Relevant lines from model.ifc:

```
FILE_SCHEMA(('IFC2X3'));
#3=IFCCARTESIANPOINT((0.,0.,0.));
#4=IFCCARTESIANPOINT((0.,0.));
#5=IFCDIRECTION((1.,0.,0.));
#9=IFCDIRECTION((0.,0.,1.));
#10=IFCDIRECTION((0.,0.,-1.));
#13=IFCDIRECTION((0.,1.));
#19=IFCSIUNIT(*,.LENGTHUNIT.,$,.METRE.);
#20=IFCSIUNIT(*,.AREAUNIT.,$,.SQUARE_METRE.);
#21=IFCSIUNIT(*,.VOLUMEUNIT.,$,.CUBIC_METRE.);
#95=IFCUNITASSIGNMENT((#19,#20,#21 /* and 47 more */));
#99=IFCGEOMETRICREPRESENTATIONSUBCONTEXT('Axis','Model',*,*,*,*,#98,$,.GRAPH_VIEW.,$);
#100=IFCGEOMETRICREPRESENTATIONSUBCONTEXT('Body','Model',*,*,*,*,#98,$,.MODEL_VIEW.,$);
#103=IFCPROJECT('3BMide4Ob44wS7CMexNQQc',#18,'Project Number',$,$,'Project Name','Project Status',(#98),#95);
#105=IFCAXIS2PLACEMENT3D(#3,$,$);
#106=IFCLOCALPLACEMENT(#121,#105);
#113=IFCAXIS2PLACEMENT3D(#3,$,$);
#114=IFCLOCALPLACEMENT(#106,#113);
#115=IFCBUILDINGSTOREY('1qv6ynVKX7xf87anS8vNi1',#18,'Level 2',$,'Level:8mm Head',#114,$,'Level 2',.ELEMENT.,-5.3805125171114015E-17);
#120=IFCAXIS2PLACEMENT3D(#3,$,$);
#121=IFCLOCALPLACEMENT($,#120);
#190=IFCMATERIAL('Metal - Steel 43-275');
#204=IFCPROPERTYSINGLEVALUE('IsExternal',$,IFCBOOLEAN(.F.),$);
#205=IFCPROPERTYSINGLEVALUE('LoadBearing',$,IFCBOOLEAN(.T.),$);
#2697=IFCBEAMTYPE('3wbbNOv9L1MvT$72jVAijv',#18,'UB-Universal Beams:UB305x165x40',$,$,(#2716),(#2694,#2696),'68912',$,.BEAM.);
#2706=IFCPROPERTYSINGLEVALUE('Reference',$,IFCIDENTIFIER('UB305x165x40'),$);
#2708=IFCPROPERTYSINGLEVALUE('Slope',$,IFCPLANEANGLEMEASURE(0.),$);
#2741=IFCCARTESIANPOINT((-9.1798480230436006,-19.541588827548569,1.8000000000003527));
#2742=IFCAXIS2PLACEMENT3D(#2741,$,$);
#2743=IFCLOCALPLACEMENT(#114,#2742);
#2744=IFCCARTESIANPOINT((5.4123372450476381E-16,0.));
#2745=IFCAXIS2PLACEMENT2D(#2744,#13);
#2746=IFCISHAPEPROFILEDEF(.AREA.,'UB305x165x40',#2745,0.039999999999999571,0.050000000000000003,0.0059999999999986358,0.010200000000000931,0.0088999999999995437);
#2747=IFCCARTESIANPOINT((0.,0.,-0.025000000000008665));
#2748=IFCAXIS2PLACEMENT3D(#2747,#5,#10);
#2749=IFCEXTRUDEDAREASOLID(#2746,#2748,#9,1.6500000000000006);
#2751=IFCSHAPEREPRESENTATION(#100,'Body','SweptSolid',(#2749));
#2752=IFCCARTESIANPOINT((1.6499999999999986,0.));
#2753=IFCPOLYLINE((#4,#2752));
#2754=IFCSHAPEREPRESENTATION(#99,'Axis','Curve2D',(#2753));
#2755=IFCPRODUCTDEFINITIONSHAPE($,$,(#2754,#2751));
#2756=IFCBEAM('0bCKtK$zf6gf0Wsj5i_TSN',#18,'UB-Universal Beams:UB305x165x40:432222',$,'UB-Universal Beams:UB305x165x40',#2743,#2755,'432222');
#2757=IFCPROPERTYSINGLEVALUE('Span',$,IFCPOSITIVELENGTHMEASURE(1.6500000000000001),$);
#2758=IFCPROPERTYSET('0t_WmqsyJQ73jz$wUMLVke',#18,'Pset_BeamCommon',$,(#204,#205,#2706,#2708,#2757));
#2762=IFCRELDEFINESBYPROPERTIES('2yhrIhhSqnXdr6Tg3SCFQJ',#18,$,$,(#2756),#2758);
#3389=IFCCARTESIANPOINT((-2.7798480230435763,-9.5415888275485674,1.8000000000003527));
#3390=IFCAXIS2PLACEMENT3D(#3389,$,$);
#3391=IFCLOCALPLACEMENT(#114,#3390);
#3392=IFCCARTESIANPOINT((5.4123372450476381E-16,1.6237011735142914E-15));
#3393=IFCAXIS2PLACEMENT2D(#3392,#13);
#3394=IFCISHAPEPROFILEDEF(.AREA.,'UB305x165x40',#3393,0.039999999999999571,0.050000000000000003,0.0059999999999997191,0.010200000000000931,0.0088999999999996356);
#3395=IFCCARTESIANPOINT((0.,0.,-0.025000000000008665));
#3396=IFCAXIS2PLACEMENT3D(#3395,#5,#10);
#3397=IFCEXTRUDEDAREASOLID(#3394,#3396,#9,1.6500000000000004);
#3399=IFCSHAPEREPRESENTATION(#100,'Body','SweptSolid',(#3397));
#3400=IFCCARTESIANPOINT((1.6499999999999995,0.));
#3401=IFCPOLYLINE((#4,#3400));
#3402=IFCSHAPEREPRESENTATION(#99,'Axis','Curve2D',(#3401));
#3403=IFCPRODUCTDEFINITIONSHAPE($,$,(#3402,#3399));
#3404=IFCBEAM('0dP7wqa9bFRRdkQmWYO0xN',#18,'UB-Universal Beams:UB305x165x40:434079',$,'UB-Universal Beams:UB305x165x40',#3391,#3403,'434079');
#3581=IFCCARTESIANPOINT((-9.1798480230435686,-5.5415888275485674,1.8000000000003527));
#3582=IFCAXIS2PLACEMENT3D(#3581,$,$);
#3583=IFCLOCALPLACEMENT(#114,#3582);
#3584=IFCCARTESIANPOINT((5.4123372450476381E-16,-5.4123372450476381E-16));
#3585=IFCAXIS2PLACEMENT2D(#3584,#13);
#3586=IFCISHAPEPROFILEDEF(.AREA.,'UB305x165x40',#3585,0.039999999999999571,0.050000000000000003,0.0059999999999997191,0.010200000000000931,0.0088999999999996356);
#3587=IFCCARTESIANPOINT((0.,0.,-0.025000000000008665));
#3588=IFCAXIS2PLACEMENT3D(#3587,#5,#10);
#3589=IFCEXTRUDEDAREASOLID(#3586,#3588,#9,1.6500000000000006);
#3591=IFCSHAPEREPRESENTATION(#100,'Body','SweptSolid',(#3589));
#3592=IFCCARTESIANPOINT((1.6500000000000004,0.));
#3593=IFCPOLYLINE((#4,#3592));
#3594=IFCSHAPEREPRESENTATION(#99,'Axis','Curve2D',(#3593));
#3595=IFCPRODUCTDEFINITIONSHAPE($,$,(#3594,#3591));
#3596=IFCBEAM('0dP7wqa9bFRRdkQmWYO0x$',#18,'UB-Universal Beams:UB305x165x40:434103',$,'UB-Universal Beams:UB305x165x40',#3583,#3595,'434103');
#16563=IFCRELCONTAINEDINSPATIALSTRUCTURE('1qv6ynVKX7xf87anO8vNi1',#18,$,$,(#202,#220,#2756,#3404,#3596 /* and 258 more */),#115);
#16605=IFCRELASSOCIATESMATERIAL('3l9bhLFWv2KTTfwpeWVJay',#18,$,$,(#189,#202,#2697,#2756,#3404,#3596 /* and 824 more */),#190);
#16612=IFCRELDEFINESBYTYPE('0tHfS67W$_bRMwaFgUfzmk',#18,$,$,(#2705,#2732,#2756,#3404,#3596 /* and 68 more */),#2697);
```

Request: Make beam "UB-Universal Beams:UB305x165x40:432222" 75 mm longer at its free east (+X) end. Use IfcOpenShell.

```python
import numpy as np
import ifcopenshell
import ifcopenshell.api.pset
import ifcopenshell.util.element
import ifcopenshell.util.representation
import ifcopenshell.util.unit

model = ifcopenshell.open("model.ifc")
unit_scale = ifcopenshell.util.unit.calculate_unit_scale(model)

member = model.by_guid("0bCKtK$zf6gf0Wsj5i_TSN")
change = 0.075 / unit_scale

# The extrusion runs towards the end named, so only its depth changes.
body = ifcopenshell.util.representation.get_representation(member, "Model", "Body")
solid = body.Items[0]
old_length = solid.Depth
solid.Depth += change

# Move the axis end point with it.
axis = next(r for r in member.Representation.Representations if r.RepresentationIdentifier == "Axis").Items[0]
start, end = (np.array(p.Coordinates) for p in axis.Points)
end = end + (end - start) / np.linalg.norm(end - start) * change
point = model.createIfcCartesianPoint(end.tolist())
axis.Points = [axis.Points[0], point]

# Update the stored length and volume.
pset = model.by_id(ifcopenshell.util.element.get_pset(member, "Pset_BeamCommon", should_inherit=False)["id"])
ifcopenshell.api.pset.edit_pset(model, pset=pset, properties={
    "Span": model.create_entity("IfcPositiveLengthMeasure", solid.Depth),
})

print(f"length {old_length:g} -> {solid.Depth:g}")

model.write("model_edited.ifc")
```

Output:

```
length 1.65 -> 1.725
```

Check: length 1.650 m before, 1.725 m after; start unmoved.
